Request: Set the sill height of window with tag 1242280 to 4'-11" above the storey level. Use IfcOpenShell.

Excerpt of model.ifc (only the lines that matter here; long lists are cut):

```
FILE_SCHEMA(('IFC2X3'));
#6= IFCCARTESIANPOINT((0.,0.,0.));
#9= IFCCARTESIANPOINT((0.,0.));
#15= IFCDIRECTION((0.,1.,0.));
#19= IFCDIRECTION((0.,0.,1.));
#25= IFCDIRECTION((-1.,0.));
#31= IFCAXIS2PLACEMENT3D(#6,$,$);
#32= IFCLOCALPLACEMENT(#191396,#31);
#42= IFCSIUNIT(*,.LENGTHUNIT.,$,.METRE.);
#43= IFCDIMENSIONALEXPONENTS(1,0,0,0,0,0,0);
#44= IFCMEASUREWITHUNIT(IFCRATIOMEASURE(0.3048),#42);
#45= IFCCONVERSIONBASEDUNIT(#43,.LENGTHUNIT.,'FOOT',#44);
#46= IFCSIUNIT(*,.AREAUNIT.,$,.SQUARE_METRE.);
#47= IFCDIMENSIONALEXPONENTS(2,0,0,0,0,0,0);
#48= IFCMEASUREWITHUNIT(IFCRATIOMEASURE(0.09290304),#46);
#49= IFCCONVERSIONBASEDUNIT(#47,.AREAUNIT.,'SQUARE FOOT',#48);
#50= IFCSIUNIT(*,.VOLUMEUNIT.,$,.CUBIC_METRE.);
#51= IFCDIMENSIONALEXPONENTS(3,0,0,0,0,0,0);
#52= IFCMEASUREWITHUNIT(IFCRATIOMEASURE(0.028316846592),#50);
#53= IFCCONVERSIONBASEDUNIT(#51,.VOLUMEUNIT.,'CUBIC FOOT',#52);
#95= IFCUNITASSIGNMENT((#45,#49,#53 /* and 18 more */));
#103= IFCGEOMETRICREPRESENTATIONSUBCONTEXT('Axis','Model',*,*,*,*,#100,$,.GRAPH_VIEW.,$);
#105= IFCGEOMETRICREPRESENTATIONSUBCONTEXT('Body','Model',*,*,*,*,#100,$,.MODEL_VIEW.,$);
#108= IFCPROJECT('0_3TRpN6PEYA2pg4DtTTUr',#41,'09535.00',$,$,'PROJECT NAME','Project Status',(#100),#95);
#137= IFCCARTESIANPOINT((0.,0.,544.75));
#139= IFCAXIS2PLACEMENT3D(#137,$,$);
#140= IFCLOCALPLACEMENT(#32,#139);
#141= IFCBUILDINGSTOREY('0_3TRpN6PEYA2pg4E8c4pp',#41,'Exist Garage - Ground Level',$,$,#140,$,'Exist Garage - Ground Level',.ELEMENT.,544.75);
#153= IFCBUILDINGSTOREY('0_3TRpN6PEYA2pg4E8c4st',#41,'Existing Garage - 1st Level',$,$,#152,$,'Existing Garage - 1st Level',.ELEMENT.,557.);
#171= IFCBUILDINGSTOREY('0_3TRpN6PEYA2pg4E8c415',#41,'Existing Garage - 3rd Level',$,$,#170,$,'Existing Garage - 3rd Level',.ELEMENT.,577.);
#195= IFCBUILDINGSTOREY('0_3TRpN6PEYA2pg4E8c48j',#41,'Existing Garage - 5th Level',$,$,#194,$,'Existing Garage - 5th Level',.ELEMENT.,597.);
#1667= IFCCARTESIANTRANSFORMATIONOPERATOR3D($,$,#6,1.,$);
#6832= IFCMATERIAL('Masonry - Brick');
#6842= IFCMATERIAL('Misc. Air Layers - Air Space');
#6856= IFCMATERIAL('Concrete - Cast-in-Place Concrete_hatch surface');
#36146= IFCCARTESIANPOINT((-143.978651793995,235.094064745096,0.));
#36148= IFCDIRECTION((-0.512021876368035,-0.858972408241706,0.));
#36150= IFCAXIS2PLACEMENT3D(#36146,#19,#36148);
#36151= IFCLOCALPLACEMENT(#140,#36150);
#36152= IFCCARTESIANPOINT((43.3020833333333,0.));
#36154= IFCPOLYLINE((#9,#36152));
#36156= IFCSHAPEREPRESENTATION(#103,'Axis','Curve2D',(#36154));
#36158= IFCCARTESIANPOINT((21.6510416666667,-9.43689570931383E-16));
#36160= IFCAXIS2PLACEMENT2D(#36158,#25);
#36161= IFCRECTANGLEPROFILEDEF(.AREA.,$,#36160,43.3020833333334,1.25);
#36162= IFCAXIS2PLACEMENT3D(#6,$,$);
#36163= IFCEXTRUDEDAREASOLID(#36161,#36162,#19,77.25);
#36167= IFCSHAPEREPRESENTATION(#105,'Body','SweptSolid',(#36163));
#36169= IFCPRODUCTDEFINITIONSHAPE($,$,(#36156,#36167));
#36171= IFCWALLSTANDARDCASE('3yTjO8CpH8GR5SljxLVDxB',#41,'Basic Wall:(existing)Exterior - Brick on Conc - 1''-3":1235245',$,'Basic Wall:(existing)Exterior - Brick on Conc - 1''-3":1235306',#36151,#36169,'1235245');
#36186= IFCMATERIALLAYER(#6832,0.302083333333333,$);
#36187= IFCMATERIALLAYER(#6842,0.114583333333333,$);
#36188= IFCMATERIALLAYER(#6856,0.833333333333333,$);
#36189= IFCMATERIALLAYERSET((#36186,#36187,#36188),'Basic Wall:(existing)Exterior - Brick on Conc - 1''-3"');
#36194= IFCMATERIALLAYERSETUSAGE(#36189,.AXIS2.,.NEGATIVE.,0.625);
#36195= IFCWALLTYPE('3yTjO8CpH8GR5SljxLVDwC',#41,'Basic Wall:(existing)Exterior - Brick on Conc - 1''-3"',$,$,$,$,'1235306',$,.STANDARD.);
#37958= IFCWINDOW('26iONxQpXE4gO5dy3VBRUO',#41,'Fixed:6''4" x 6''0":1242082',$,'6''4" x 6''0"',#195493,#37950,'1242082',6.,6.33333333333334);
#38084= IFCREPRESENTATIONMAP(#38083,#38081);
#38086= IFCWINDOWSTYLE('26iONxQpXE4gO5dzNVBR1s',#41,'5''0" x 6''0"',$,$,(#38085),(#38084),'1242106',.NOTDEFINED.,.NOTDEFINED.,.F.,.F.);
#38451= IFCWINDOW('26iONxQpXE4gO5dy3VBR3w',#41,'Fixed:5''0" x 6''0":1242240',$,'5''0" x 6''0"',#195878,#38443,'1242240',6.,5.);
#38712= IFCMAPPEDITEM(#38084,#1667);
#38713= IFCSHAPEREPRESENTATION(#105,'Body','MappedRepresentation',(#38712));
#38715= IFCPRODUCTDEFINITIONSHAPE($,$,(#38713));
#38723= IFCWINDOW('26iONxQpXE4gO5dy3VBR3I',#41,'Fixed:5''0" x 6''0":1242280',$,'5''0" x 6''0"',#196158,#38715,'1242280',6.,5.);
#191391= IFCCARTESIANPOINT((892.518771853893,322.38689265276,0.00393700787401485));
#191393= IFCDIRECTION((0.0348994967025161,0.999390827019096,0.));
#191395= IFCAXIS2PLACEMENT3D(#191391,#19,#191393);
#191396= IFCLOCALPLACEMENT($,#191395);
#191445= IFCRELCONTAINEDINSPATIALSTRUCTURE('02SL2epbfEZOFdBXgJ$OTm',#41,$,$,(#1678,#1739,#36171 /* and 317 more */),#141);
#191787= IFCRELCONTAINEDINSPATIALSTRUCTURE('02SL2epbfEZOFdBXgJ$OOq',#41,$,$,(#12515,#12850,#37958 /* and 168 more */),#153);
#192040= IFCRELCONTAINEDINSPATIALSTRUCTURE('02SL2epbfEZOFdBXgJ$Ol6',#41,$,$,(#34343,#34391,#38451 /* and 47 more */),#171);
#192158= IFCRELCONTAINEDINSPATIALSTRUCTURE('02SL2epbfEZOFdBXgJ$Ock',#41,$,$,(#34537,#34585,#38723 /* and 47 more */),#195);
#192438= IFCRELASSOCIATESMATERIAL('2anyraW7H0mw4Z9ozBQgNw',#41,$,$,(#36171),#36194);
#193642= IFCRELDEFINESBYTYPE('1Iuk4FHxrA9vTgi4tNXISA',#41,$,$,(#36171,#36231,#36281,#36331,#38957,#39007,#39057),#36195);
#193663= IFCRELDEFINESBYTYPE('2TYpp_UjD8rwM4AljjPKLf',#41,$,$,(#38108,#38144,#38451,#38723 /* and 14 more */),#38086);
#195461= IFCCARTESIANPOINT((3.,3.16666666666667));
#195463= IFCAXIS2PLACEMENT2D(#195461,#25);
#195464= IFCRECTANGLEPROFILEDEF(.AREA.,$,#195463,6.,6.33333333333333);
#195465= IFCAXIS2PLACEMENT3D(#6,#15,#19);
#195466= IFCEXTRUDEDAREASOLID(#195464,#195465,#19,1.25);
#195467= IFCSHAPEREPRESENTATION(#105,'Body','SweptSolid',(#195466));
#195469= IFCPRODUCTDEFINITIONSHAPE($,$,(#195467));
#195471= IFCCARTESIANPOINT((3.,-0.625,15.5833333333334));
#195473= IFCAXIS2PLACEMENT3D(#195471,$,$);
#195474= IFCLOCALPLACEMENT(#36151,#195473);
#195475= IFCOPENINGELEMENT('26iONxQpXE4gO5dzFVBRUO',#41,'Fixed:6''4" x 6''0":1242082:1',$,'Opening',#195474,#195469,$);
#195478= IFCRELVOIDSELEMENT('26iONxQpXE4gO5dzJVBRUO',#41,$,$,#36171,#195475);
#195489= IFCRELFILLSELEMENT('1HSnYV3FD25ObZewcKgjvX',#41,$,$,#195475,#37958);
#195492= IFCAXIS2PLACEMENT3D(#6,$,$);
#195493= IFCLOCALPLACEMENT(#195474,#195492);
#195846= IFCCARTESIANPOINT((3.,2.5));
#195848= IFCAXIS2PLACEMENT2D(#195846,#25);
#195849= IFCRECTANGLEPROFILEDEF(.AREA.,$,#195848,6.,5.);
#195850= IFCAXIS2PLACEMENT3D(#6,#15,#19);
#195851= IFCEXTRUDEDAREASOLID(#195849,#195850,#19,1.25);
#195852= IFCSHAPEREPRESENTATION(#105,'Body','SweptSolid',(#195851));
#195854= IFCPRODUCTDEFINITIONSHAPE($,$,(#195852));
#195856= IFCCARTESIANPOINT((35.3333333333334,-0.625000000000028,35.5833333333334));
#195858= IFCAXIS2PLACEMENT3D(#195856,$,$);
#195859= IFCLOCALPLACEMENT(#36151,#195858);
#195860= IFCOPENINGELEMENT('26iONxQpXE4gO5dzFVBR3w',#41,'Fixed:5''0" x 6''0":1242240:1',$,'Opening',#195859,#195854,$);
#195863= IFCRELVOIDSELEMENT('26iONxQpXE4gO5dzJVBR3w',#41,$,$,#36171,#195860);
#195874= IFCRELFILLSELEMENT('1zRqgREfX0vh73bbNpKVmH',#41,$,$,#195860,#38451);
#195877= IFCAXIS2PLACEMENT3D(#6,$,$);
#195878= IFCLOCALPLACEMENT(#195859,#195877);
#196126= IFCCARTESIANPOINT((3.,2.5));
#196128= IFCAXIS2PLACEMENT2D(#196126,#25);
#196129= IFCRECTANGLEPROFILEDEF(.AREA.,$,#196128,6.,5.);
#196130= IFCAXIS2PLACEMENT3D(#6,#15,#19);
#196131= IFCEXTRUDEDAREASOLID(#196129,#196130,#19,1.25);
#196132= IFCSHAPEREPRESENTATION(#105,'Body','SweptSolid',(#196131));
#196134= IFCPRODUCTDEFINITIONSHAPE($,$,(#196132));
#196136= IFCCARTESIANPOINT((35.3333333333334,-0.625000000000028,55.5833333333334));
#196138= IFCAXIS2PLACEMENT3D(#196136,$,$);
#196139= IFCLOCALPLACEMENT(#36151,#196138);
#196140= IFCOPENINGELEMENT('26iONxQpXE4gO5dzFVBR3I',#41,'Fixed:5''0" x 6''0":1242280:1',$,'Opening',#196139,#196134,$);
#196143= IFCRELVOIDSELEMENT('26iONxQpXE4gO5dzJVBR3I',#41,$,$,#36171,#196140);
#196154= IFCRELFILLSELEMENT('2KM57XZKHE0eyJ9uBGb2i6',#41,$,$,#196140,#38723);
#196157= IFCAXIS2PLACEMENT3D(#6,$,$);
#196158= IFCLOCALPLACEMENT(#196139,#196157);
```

```python
import numpy as np
import ifcopenshell
import ifcopenshell.api.geometry
import ifcopenshell.geom
import ifcopenshell.util.element
import ifcopenshell.util.placement
import ifcopenshell.util.shape
import ifcopenshell.util.unit

model = ifcopenshell.open("model.ifc")
unit_scale = ifcopenshell.util.unit.calculate_unit_scale(model)

window = model.by_guid("26iONxQpXE4gO5dy3VBR3I")
opening = window.FillsVoids[0].RelatingOpeningElement
storey = ifcopenshell.util.element.get_container(window, ifc_class="IfcBuildingStorey")
level = ifcopenshell.util.placement.get_local_placement(storey.ObjectPlacement)[2, 3]

# The opening's origin need not be at the sill, so measure its lowest point.
shape = ifcopenshell.geom.create_shape(ifcopenshell.geom.settings(), opening)
bottom = ifcopenshell.util.shape.get_shape_bottom_elevation(shape, shape.geometry) / unit_scale
dz = level + 59 * 0.0254 / unit_scale - bottom

shift = np.array([0.0, 0.0, dz])
# The window is placed relative to its opening, so it follows when the opening moves.
matrix = ifcopenshell.util.placement.get_local_placement(opening.ObjectPlacement)
matrix[:3, 3] += shift
ifcopenshell.api.geometry.edit_object_placement(
    model, product=opening, matrix=matrix, is_si=False, should_transform_children=True
)

print(f"moved by {dz * unit_scale:+.3f} m")

model.write("model_rev.ifc")
```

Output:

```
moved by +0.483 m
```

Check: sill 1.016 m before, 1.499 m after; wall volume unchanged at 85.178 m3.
